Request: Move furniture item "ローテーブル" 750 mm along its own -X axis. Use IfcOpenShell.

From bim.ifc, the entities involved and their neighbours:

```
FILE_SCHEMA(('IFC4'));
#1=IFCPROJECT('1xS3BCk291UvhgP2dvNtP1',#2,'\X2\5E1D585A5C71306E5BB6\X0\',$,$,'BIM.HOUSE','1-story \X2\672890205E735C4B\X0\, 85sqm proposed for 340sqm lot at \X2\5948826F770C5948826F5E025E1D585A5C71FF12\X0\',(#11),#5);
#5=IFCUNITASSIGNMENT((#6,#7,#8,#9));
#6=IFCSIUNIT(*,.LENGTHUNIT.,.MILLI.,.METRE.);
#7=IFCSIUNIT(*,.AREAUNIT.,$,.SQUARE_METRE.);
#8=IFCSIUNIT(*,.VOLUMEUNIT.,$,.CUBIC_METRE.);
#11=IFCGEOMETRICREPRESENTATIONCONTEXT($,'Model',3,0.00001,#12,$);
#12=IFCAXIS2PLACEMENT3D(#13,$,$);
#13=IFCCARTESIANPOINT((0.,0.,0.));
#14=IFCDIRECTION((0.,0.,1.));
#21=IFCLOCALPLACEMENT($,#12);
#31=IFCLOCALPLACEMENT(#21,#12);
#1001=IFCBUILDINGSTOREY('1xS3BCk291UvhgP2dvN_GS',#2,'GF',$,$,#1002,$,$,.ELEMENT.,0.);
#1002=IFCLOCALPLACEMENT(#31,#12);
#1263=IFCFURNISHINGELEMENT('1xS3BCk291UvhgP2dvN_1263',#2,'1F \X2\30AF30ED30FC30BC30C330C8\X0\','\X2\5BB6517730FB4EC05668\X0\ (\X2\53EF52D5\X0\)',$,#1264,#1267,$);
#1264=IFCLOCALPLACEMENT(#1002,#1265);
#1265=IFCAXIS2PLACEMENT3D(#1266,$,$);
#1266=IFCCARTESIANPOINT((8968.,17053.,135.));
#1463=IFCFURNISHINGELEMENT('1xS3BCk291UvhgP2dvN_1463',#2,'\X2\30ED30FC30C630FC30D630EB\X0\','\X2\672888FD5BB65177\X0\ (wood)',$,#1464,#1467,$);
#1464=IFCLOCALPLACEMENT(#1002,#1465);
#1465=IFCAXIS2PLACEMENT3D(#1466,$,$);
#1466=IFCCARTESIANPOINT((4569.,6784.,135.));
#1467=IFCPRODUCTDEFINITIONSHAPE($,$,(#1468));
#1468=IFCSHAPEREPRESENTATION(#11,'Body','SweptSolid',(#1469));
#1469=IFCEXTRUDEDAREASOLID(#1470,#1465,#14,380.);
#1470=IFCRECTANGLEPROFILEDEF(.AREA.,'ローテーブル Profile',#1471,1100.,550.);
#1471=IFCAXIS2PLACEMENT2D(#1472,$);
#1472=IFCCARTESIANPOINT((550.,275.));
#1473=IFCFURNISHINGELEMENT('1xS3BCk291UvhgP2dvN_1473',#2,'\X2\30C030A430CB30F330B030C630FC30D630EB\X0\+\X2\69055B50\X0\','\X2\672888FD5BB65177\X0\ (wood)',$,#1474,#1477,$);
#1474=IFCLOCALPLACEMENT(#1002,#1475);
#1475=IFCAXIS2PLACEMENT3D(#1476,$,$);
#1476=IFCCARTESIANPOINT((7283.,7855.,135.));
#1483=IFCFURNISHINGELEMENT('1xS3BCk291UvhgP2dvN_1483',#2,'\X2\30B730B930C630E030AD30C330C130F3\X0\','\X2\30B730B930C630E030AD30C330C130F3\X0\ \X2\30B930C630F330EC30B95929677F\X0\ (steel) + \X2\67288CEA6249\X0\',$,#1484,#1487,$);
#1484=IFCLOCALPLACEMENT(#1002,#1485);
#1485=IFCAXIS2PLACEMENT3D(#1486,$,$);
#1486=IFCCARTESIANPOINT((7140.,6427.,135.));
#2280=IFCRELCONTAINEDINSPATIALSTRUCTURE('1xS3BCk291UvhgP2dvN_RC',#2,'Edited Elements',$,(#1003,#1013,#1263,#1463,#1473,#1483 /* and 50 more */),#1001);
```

```python
import ifcopenshell
import ifcopenshell.api.geometry
import ifcopenshell.util.placement

model = ifcopenshell.open("bim.ifc")

item = model.by_id(1463)
matrix = ifcopenshell.util.placement.get_local_placement(item.ObjectPlacement)
matrix[:3, 3] -= matrix[:3, 0] * 750.0
ifcopenshell.api.geometry.edit_object_placement(model, product=item, matrix=matrix, is_si=False)

print(ifcopenshell.util.placement.get_local_placement(item.ObjectPlacement).round(3) + 0.0)

model.write("bim_v2.ifc")
```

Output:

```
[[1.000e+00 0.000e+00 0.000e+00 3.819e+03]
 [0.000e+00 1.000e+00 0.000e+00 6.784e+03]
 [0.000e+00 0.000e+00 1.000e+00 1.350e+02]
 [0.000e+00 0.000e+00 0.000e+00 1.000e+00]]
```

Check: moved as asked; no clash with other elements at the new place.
